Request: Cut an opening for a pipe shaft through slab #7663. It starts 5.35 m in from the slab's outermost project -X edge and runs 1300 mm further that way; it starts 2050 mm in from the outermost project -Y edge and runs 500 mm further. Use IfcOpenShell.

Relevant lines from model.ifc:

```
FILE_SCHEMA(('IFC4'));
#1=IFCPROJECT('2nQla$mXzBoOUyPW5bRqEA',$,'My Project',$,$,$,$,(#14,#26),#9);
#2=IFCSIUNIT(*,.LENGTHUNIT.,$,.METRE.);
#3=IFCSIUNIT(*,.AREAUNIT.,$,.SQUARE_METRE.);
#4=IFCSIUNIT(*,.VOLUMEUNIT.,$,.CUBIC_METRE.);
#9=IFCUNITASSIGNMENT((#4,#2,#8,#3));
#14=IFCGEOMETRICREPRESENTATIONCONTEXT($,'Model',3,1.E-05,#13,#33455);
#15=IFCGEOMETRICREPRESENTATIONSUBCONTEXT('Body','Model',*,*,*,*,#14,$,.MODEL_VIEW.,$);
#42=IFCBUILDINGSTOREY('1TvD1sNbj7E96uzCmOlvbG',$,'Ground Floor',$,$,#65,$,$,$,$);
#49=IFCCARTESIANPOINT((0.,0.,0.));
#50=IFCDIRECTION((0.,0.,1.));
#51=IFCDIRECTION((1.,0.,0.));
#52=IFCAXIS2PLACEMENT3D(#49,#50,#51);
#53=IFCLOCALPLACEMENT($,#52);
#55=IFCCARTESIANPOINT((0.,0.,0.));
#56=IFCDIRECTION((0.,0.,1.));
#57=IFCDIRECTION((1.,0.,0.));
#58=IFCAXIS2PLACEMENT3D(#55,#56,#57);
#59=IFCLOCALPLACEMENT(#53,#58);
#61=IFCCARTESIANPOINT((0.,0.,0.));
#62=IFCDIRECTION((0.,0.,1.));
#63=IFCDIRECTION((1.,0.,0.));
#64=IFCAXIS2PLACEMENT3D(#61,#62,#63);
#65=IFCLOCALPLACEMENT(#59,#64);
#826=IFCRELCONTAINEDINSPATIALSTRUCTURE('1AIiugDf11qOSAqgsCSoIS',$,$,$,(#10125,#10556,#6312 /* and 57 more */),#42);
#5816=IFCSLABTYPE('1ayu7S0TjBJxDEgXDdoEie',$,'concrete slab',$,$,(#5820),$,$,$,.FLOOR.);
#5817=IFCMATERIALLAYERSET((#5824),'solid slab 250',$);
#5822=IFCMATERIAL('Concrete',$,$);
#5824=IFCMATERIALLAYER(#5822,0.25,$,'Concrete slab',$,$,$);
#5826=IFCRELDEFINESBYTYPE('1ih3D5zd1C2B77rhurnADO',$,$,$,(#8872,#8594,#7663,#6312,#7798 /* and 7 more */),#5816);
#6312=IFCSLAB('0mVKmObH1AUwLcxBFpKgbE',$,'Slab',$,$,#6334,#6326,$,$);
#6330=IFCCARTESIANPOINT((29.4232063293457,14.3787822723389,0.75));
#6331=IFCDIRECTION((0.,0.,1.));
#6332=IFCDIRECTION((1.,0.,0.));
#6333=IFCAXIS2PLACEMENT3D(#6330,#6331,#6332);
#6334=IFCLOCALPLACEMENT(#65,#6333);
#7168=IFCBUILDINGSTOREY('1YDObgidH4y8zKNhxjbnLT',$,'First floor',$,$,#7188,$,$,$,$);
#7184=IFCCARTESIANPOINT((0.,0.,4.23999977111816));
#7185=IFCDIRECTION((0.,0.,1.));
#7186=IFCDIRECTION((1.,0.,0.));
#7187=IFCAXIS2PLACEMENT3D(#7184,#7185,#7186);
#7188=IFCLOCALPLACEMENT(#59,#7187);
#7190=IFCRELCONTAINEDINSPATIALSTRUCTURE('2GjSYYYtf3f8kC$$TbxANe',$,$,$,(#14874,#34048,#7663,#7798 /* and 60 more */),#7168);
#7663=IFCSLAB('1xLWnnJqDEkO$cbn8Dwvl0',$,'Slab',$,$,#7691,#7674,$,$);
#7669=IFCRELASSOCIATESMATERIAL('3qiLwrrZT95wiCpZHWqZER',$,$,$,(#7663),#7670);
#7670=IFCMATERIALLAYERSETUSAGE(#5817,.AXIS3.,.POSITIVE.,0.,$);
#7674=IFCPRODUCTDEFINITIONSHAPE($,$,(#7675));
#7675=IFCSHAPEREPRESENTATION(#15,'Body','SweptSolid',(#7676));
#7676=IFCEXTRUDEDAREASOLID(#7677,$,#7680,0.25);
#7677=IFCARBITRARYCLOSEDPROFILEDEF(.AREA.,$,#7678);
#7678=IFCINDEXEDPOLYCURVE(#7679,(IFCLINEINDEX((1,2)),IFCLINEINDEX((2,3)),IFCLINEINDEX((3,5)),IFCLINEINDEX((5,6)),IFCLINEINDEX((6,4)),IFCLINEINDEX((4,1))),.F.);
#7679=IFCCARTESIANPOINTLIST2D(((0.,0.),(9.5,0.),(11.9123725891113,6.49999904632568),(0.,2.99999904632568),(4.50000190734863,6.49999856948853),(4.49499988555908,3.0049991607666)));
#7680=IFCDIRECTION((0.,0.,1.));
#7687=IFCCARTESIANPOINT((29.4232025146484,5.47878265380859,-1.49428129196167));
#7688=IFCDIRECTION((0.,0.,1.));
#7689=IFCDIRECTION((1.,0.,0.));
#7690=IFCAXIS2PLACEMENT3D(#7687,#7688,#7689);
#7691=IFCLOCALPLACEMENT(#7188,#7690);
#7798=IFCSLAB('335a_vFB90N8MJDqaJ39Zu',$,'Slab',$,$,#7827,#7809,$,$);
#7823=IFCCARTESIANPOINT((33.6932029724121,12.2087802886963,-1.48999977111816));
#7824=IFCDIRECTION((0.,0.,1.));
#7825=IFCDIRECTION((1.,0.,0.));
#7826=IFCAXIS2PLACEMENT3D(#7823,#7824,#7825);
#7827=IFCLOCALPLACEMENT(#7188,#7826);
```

```python
import numpy as np
import ifcopenshell
import ifcopenshell.api.feature
import ifcopenshell.api.geometry
import ifcopenshell.api.root
import ifcopenshell.geom
import ifcopenshell.util.placement
import ifcopenshell.util.representation
import ifcopenshell.util.shape
import ifcopenshell.util.unit

model = ifcopenshell.open("model.ifc")
unit_scale = ifcopenshell.util.unit.calculate_unit_scale(model)
settings = ifcopenshell.geom.settings()


def volume(element):
    """Net volume in cubic metres, openings subtracted."""
    shape = ifcopenshell.geom.create_shape(settings, element)
    return ifcopenshell.util.shape.get_volume(shape.geometry)


slab = model.by_guid("1xLWnnJqDEkO$cbn8Dwvl0")
before = volume(slab)

# Extent in the slab's own axes, in metres. The edges named are its -X and -Y sides.
slab_shape = ifcopenshell.geom.create_shape(settings, slab)
vertices = ifcopenshell.util.shape.get_vertices(slab_shape.geometry)
x_min, y_min, bottom = vertices.min(axis=0)
top = vertices[:, 2].max()

opening = ifcopenshell.api.root.create_entity(model, ifc_class="IfcOpeningElement", name="Pipe shaft opening", predefined_type="OPENING")
context = ifcopenshell.util.representation.get_context(model, "Model", "Body", "MODEL_VIEW")
width, depth = 1.3, 0.5
outline = [(0.0, 0.0), (width, 0.0), (width, depth), (0.0, depth), (0.0, 0.0)]
# Overshoot both faces by 50 mm so the cut is clean.
shape = ifcopenshell.api.geometry.add_slab_representation(
    model, context=context, depth=top - bottom + 0.1, polyline=outline
)
ifcopenshell.api.geometry.assign_representation(model, product=opening, representation=shape)

matrix = ifcopenshell.util.placement.get_local_placement(slab.ObjectPlacement)
matrix[:, 3] = matrix @ np.append(np.array([x_min + 5.35, y_min + 2.05, bottom - 0.05]) / unit_scale, 1.0)
ifcopenshell.api.geometry.edit_object_placement(model, product=opening, matrix=matrix, is_si=False)
ifcopenshell.api.feature.add_feature(model, feature=opening, element=slab)

after = volume(slab)

print(f"slab volume {before:.3f} -> {after:.3f} m3")

model.write("model_v2.ifc")
```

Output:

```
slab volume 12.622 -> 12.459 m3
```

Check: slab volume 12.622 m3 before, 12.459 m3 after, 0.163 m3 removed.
